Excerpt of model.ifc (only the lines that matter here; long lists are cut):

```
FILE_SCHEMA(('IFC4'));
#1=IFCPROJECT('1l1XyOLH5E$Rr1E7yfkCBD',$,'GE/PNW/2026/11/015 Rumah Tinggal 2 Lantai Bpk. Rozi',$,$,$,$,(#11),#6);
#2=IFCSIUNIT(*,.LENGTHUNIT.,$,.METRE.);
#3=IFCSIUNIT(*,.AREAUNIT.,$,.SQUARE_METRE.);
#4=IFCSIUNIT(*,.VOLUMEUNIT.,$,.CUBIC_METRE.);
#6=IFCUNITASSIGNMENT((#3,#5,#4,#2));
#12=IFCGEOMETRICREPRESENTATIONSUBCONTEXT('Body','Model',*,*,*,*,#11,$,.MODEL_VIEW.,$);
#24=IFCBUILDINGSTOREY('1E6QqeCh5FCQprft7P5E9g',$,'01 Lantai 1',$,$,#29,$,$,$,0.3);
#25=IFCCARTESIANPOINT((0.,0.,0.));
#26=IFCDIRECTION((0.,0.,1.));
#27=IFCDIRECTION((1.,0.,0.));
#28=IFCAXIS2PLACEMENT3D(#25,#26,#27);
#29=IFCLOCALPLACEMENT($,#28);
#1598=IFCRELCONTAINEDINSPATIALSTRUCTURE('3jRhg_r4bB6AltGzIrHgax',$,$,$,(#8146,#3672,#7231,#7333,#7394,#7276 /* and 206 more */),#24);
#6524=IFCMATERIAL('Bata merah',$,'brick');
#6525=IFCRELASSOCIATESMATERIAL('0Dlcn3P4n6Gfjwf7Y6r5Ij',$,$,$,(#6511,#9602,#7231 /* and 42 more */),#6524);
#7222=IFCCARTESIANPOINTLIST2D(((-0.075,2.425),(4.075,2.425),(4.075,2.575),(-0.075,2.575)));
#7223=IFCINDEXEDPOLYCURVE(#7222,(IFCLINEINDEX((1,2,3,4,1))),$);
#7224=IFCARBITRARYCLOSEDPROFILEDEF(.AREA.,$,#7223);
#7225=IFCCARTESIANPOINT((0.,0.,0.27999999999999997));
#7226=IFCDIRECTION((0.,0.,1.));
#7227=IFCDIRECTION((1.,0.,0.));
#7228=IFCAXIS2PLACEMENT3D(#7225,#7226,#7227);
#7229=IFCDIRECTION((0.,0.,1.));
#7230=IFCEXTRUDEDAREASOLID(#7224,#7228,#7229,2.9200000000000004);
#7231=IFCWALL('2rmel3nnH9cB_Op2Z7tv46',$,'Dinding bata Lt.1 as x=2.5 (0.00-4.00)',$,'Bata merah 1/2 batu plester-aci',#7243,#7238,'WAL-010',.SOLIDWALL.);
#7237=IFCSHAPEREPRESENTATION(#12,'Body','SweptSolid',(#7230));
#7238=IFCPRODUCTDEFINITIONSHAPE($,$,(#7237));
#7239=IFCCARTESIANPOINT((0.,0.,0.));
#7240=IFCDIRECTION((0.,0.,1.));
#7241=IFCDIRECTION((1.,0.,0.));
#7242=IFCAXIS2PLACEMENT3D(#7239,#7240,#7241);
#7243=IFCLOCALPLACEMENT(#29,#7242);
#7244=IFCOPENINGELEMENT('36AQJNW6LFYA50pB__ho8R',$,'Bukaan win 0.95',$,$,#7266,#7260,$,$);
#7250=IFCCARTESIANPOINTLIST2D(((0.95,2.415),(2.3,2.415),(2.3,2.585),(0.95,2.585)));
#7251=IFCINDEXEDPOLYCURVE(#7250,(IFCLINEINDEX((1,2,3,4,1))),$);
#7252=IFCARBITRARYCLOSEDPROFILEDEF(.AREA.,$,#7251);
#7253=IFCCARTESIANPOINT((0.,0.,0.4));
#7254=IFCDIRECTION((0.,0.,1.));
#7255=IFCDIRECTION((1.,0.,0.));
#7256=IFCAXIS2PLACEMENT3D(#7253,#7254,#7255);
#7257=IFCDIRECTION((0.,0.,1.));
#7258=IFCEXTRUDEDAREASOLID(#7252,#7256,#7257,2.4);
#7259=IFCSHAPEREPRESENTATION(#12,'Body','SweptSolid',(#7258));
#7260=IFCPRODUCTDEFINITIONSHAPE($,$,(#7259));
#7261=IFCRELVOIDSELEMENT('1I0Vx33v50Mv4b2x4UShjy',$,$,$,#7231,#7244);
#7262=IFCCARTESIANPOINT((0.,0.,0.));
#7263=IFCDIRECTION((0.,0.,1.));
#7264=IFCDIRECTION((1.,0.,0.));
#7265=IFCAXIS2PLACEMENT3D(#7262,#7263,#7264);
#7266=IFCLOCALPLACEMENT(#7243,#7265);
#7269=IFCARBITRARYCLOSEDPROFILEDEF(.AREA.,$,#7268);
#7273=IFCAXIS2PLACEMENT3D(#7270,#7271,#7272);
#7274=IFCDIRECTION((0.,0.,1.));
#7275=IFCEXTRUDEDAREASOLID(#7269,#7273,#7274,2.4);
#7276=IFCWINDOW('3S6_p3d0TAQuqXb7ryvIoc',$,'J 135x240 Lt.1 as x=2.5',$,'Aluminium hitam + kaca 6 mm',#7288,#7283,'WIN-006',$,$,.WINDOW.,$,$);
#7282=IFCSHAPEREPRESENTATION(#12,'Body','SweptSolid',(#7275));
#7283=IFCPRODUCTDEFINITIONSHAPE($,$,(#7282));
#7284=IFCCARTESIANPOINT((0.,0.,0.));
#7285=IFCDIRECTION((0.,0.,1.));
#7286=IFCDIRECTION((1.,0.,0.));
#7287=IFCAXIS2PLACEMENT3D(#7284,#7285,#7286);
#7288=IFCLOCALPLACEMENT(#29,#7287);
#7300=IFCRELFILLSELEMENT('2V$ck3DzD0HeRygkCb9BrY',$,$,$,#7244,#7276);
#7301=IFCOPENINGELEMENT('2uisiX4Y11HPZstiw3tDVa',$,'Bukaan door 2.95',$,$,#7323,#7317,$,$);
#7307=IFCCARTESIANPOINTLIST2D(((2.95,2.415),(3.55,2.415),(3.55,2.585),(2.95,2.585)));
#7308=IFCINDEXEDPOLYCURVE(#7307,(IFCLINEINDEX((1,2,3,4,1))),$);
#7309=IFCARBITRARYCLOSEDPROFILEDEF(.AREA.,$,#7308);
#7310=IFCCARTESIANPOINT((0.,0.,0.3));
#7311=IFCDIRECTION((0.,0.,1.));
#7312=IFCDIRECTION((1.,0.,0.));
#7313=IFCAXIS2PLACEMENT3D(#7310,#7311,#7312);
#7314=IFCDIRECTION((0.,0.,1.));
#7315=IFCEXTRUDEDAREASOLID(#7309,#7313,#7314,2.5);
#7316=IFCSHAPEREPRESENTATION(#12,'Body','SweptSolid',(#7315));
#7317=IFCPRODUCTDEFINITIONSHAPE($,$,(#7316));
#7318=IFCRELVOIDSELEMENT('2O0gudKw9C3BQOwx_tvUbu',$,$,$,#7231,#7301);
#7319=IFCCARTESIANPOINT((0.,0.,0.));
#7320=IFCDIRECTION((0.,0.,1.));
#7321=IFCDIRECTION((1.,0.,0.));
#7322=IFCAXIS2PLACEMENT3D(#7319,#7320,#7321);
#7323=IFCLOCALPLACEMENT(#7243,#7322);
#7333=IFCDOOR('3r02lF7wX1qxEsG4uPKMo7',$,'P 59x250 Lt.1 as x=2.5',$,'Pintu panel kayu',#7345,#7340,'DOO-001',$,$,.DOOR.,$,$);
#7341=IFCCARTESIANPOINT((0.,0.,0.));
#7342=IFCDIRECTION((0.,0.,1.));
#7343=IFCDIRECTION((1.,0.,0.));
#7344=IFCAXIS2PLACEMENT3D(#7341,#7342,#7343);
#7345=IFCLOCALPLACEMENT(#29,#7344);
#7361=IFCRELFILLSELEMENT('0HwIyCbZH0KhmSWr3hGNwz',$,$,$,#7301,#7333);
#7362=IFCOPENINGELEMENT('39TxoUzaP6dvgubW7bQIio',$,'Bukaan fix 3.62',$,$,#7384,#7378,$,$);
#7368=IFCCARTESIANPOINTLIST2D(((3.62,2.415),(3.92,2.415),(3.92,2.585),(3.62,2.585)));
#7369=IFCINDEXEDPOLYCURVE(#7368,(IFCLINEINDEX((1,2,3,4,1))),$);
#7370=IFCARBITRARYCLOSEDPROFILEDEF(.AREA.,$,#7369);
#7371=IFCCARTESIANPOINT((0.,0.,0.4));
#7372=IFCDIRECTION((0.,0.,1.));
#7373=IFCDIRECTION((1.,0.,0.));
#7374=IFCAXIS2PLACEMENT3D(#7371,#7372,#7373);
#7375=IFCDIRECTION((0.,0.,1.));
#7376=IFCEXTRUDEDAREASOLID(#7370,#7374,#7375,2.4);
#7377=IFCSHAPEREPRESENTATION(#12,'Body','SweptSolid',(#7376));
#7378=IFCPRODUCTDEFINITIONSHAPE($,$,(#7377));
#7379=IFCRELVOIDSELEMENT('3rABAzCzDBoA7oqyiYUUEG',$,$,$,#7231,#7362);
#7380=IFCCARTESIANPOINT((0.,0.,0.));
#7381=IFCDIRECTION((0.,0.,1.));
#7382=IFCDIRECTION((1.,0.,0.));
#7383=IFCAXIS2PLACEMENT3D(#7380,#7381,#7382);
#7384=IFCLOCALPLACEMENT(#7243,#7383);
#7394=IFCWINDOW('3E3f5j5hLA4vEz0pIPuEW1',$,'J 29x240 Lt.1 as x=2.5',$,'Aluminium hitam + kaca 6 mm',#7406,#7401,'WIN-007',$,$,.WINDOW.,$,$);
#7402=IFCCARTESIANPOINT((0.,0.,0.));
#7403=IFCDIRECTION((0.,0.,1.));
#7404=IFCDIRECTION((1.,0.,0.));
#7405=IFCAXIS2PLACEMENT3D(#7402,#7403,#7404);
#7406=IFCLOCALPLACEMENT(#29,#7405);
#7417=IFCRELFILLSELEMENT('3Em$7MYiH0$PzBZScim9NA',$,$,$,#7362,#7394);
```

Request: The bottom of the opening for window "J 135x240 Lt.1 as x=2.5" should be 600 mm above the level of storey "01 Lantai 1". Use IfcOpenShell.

```python
import numpy as np
import ifcopenshell
import ifcopenshell.api.geometry
import ifcopenshell.geom
import ifcopenshell.util.element
import ifcopenshell.util.placement
import ifcopenshell.util.shape
import ifcopenshell.util.unit

model = ifcopenshell.open("model.ifc")
unit_scale = ifcopenshell.util.unit.calculate_unit_scale(model)

window = model.by_id(7276)
opening = window.FillsVoids[0].RelatingOpeningElement
storey = ifcopenshell.util.element.get_container(window, ifc_class="IfcBuildingStorey")
level = ifcopenshell.util.placement.get_local_placement(storey.ObjectPlacement)[2, 3]

# The opening's origin need not be at the sill, so measure its lowest point.
shape = ifcopenshell.geom.create_shape(ifcopenshell.geom.settings(), opening)
bottom = ifcopenshell.util.shape.get_shape_bottom_elevation(shape, shape.geometry) / unit_scale
dz = level + 0.6 / unit_scale - bottom

shift = np.array([0.0, 0.0, dz])
# The window is not placed relative to its opening, so move both.
for product in (opening, window):
    matrix = ifcopenshell.util.placement.get_local_placement(product.ObjectPlacement)
    matrix[:3, 3] += shift
    ifcopenshell.api.geometry.edit_object_placement(model, product=product, matrix=matrix, is_si=False)

print(f"moved by {dz * unit_scale:+.3f} m")

model.write("model_v2.ifc")
```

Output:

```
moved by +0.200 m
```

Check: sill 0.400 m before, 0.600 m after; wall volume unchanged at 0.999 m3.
